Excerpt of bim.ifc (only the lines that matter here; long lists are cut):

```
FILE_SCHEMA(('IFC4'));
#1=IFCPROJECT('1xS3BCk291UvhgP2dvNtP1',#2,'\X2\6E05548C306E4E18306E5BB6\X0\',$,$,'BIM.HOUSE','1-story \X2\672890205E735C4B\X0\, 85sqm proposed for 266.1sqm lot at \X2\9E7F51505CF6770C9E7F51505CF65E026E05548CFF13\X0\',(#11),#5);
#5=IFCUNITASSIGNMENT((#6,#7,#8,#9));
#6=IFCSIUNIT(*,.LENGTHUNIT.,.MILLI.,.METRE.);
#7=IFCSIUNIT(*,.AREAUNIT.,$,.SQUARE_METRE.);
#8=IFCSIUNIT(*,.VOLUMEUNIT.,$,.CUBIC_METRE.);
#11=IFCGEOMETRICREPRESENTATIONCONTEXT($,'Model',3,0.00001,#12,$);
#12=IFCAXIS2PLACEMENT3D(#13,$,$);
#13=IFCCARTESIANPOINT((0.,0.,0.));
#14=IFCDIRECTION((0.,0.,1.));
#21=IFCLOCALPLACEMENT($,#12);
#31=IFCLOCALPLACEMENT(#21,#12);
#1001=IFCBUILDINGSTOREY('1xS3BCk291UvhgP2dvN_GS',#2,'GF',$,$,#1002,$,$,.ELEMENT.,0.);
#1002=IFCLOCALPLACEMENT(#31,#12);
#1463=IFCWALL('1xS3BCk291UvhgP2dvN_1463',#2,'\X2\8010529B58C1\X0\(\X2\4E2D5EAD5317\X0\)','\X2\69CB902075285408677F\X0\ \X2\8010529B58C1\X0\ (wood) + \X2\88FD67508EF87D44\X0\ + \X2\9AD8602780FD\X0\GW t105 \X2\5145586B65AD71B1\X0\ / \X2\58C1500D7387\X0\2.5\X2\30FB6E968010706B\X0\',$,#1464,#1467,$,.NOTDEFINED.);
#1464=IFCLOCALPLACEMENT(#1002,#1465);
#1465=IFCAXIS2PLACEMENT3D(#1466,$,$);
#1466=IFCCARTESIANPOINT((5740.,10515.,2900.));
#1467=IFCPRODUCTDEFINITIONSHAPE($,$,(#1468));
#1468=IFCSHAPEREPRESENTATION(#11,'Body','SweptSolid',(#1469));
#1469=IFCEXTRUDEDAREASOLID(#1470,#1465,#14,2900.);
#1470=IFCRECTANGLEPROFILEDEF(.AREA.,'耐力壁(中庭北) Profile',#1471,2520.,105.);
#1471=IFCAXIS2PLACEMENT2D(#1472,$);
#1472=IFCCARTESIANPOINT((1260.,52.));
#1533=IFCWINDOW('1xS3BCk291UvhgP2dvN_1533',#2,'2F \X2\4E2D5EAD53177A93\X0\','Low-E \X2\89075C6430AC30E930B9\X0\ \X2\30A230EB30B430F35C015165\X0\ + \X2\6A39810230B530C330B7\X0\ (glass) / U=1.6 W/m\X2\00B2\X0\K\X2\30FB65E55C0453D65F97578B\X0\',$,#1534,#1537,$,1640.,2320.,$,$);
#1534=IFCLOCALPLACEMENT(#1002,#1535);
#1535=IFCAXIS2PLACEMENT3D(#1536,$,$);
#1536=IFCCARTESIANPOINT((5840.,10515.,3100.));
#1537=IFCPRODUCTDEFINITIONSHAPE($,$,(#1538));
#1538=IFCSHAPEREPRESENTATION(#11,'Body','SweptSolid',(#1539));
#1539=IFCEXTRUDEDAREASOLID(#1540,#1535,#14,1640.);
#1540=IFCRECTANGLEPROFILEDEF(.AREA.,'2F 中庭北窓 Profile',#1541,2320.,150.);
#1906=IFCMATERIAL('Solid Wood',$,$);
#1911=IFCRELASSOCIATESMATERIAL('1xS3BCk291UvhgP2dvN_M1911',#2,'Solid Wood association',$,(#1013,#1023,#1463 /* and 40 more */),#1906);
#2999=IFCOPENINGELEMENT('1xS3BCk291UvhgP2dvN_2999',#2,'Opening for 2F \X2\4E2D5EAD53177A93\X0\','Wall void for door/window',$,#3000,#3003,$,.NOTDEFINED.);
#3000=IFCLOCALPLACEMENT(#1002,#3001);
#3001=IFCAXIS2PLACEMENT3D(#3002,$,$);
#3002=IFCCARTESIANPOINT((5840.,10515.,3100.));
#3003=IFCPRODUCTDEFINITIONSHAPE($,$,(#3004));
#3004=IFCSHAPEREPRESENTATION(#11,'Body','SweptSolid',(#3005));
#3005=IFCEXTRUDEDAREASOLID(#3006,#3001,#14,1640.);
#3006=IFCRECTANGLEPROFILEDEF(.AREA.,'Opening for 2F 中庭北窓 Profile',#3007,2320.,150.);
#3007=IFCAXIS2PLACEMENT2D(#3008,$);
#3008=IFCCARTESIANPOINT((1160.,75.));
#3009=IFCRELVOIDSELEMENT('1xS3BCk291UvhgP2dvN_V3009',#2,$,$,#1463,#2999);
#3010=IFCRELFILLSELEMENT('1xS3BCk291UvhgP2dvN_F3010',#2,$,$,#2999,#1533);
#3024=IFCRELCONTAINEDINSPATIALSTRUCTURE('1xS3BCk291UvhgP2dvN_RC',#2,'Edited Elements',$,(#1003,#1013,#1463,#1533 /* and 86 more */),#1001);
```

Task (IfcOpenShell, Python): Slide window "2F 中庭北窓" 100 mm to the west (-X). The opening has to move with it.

```python
import ifcopenshell
import ifcopenshell.api.geometry
import ifcopenshell.util.placement

model = ifcopenshell.open("bim.ifc")

window = model.by_guid("1xS3BCk291UvhgP2dvN_1533")
opening = window.FillsVoids[0].RelatingOpeningElement
wall = opening.VoidsElements[0].RelatingBuildingElement

wall_matrix = ifcopenshell.util.placement.get_local_placement(wall.ObjectPlacement)
shift = wall_matrix[:3, 0] * -100.0
before = ifcopenshell.util.placement.get_local_placement(window.ObjectPlacement)[:3, 3].copy()

# The window is not placed relative to its opening, so move both.
for product in (opening, window):
    matrix = ifcopenshell.util.placement.get_local_placement(product.ObjectPlacement)
    matrix[:3, 3] += shift
    ifcopenshell.api.geometry.edit_object_placement(model, product=product, matrix=matrix, is_si=False)

after = ifcopenshell.util.placement.get_local_placement(window.ObjectPlacement)[:3, 3]
print("window moved by", (after - before).round(3) + 0.0)

model.write("bim_v2.ifc")
```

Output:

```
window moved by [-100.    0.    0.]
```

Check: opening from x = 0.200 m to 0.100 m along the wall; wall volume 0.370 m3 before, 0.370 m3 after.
